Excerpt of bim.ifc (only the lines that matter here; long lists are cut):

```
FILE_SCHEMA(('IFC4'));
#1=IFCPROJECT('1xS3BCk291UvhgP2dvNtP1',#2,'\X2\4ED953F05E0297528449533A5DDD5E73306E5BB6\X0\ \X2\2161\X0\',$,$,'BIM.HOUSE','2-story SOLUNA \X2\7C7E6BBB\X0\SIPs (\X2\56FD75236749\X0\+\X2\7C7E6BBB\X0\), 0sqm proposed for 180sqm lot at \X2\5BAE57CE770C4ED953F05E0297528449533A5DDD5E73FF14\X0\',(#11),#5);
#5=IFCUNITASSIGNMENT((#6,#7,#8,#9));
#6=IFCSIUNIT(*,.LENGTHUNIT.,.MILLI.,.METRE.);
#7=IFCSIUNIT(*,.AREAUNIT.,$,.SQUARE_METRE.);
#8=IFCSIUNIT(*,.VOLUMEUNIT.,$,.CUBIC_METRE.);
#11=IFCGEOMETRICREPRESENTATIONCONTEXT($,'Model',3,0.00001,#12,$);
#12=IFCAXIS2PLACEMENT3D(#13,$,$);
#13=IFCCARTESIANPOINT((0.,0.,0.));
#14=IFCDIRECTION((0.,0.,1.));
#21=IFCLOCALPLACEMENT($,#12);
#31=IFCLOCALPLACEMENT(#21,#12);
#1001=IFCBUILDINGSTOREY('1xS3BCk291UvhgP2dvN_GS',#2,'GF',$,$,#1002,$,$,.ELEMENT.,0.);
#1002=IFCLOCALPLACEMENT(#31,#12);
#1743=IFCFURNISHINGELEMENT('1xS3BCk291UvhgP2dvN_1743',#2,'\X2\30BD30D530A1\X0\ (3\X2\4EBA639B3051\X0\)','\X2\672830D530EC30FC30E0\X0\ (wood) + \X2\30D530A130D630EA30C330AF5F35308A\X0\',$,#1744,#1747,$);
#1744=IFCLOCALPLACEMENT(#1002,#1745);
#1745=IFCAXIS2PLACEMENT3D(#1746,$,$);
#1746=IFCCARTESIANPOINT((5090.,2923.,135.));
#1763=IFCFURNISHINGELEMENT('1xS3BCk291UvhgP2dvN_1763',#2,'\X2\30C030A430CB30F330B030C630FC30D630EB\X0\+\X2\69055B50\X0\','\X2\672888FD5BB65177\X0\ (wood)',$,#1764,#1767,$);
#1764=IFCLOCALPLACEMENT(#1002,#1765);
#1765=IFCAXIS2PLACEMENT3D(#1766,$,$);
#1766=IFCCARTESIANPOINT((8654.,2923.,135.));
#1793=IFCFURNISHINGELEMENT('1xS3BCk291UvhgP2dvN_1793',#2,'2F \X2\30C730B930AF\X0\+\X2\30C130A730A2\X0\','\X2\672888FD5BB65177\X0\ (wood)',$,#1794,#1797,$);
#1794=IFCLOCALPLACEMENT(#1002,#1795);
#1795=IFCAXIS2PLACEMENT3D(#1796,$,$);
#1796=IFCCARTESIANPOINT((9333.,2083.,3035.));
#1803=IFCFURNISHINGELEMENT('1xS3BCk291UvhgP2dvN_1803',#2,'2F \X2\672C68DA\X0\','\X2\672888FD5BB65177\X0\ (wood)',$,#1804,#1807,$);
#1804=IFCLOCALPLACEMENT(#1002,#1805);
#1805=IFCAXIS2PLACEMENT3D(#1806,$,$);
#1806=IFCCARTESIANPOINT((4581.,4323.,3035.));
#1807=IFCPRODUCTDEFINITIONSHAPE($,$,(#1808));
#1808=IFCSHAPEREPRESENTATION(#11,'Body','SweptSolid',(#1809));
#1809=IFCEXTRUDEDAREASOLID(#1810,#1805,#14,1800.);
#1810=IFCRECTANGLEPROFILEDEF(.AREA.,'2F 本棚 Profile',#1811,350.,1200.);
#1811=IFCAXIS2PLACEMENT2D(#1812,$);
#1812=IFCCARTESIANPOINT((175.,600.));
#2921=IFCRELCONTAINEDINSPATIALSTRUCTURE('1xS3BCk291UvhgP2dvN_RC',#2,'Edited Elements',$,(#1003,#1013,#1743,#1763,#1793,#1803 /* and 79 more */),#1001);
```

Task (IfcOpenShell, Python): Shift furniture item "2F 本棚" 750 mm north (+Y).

```python
import ifcopenshell
import ifcopenshell.api.geometry
import ifcopenshell.util.placement

model = ifcopenshell.open("bim.ifc")

item = model.by_id(1803)
matrix = ifcopenshell.util.placement.get_local_placement(item.ObjectPlacement)
matrix[1, 3] += 750.0
ifcopenshell.api.geometry.edit_object_placement(model, product=item, matrix=matrix, is_si=False)

print(ifcopenshell.util.placement.get_local_placement(item.ObjectPlacement).round(3) + 0.0)

model.write("bim-out.ifc")
```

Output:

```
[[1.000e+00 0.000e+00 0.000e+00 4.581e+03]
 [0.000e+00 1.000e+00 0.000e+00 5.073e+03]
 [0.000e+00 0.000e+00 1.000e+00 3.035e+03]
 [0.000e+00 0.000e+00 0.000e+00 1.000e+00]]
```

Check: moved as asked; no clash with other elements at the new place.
